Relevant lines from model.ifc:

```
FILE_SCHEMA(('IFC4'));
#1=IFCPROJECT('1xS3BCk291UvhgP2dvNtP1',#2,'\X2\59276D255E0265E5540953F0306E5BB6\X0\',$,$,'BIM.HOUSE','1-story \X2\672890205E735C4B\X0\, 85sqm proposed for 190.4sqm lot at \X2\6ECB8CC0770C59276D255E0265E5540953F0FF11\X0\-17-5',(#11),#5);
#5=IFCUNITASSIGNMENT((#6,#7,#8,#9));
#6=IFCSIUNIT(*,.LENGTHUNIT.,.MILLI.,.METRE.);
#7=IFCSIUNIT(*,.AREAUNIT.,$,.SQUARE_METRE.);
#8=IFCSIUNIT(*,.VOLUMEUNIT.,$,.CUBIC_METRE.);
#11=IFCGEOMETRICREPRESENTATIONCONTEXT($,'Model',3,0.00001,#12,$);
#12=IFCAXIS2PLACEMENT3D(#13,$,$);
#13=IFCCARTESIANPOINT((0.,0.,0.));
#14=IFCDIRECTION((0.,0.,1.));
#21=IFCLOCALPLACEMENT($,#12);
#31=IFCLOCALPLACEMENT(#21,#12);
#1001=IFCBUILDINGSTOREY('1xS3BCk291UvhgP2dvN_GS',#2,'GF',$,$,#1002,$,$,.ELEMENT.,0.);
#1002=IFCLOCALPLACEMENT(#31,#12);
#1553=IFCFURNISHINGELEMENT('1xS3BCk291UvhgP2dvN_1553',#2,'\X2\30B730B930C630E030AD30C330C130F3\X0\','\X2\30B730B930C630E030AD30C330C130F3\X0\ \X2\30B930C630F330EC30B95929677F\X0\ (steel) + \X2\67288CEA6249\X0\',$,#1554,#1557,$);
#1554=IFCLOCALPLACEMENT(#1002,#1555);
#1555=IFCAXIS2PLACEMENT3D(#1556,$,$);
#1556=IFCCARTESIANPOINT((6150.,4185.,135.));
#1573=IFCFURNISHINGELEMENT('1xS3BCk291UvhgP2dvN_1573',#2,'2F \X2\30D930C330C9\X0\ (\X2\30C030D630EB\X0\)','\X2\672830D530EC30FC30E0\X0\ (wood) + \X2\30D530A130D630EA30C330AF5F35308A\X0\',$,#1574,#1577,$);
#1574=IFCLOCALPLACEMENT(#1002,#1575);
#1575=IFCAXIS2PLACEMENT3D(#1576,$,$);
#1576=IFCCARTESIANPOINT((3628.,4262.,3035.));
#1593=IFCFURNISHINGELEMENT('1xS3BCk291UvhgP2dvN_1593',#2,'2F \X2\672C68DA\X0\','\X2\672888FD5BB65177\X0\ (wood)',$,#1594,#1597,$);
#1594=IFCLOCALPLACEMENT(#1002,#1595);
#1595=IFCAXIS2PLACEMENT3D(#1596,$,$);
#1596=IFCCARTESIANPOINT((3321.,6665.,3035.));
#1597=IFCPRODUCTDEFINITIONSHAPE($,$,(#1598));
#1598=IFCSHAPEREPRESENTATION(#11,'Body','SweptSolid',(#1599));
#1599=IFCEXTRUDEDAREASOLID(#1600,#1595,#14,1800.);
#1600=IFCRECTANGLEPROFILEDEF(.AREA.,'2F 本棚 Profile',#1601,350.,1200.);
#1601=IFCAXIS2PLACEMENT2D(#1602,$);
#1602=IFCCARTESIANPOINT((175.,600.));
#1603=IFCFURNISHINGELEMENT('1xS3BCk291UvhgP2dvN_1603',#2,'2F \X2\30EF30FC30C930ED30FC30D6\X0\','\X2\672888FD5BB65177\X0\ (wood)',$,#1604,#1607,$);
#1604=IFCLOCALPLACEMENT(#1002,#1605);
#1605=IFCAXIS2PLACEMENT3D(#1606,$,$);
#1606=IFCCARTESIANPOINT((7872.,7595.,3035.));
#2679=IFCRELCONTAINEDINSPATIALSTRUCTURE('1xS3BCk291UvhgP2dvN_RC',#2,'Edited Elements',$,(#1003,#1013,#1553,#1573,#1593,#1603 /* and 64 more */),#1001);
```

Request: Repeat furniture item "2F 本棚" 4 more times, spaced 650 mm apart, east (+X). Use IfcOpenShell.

```python
import numpy as np
import ifcopenshell
import ifcopenshell.api.geometry
import ifcopenshell.api.root
import ifcopenshell.util.element
import ifcopenshell.util.placement
import ifcopenshell.util.unit

model = ifcopenshell.open("model.ifc")
unit_scale = ifcopenshell.util.unit.calculate_unit_scale(model)


def reuse_history(source, copy):
    """copy_class also copies each property set's owner history, people and application; keep the originals."""
    for rel in copy.IsDefinedBy:
        if rel.is_a("IfcRelDefinesByProperties") and (history := rel.RelatingPropertyDefinition.OwnerHistory):
            rel.RelatingPropertyDefinition.OwnerHistory = source.OwnerHistory
            ifcopenshell.util.element.remove_deep2(model, history)


source = model.by_id(1593)
base = ifcopenshell.util.placement.get_local_placement(source.ObjectPlacement)
step = np.array([1.0, 0.0, 0.0]) * 0.65 / unit_scale

for i in range(1, 5):
    copy = ifcopenshell.api.root.copy_class(model, product=source)
    copy.Representation = ifcopenshell.util.element.copy_deep(
        model, source.Representation, exclude=["IfcGeometricRepresentationContext", "IfcRepresentationMap"]
    )
    reuse_history(source, copy)
    matrix = base.copy()
    matrix[:3, 3] += i * step
    print("added at", matrix[:3, 3].round(3) + 0.0)
    ifcopenshell.api.geometry.edit_object_placement(model, product=copy, matrix=matrix, is_si=False)

model.write("model-out.ifc")
```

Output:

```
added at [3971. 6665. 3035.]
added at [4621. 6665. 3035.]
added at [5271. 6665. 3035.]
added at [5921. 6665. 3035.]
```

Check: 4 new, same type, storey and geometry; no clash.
